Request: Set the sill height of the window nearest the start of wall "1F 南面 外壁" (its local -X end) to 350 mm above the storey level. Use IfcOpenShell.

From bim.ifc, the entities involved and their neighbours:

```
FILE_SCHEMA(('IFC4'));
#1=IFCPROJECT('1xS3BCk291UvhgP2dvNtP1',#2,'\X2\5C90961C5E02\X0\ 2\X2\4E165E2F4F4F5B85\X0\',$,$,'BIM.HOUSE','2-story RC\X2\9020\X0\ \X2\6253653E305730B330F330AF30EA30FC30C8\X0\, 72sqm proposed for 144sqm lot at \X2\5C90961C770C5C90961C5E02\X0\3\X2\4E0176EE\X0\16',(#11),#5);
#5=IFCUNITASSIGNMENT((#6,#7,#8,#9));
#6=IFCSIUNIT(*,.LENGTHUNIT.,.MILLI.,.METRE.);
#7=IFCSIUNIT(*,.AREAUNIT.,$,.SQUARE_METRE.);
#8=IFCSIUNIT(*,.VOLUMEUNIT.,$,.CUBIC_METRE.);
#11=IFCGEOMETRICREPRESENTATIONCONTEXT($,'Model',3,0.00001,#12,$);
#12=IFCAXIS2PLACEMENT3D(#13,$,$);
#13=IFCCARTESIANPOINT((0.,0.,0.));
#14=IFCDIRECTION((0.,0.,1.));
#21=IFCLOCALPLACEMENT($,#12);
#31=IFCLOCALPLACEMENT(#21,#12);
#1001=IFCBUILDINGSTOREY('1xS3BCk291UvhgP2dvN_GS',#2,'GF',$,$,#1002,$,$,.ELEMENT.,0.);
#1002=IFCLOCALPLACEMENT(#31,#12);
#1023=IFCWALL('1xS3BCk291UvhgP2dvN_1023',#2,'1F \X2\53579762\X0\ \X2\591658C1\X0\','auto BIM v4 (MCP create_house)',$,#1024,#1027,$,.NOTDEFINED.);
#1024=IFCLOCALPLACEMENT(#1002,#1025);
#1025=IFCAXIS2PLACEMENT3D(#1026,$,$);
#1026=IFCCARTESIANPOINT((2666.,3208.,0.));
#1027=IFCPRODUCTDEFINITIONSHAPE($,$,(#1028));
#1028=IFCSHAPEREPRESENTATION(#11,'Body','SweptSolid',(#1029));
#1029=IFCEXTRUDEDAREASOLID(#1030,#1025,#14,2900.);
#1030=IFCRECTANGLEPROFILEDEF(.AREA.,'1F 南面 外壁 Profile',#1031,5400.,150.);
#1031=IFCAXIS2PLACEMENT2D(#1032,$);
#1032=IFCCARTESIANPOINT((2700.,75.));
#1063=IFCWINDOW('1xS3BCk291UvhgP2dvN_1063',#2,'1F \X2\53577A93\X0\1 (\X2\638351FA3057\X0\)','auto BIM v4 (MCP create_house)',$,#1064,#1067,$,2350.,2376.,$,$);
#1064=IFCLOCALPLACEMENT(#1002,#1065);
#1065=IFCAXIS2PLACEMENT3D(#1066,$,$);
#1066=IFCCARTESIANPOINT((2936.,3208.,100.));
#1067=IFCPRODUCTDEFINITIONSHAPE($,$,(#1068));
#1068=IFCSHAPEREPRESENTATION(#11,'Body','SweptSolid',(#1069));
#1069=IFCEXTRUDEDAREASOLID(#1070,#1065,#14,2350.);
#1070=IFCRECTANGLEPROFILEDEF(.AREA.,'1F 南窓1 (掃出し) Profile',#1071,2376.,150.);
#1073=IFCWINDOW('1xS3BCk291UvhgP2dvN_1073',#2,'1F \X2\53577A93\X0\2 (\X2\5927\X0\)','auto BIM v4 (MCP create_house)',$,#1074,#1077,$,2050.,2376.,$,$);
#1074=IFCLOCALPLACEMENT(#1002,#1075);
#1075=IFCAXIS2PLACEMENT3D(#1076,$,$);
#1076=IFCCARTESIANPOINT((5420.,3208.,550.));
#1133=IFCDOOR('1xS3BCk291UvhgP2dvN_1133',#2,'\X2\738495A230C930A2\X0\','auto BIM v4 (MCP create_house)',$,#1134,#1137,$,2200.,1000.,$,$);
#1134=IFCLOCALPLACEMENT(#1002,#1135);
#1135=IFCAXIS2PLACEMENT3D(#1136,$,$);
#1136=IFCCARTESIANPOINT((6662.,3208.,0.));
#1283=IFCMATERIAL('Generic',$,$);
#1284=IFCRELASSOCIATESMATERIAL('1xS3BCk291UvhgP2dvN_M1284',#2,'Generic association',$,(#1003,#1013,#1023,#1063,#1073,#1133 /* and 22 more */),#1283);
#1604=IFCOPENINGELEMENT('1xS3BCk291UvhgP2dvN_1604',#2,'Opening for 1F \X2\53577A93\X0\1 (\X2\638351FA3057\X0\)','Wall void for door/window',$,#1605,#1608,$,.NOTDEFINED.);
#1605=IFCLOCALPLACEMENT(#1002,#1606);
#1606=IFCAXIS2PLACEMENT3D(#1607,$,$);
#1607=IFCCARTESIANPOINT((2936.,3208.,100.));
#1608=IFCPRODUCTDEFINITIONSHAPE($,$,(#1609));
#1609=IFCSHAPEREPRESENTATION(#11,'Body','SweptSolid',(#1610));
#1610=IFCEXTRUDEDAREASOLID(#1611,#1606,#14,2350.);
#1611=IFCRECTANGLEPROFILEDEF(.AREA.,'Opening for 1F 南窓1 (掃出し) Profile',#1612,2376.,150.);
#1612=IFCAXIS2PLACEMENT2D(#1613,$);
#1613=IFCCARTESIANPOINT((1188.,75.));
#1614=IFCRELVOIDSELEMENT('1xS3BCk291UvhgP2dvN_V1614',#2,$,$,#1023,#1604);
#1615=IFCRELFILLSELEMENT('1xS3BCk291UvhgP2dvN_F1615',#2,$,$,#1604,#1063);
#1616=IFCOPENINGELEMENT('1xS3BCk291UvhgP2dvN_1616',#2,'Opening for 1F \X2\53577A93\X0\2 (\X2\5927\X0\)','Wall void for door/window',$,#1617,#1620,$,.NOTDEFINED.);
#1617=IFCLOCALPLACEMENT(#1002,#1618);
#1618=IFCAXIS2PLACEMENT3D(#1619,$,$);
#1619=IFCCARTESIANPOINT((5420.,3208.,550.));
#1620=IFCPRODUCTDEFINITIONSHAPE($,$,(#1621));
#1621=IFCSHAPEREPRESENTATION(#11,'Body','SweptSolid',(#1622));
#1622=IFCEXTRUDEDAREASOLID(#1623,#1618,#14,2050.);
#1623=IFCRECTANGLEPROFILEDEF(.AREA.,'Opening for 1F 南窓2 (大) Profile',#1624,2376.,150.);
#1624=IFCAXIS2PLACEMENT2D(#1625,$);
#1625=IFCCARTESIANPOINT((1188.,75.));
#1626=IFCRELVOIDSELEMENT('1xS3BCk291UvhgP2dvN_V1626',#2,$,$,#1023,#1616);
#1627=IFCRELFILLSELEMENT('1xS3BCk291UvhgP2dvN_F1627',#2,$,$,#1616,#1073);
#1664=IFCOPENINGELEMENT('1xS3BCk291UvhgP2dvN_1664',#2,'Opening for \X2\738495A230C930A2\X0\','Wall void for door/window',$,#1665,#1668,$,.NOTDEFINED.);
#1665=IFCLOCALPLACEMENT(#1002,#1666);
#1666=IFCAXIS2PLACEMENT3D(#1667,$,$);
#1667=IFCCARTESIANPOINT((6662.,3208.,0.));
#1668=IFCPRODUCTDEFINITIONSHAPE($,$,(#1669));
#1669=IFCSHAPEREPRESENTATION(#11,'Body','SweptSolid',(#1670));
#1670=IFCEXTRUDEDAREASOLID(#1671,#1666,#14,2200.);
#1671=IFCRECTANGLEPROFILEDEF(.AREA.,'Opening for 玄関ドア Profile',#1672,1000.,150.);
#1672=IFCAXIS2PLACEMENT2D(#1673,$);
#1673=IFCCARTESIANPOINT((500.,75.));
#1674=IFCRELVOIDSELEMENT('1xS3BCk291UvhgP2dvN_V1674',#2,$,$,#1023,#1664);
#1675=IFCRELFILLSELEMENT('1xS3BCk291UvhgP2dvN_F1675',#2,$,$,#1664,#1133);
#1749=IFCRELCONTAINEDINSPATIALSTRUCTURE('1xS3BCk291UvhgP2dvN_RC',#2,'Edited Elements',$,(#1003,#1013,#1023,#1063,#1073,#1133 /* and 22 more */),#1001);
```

```python
import numpy as np
import ifcopenshell
import ifcopenshell.api.geometry
import ifcopenshell.geom
import ifcopenshell.util.element
import ifcopenshell.util.placement
import ifcopenshell.util.shape
import ifcopenshell.util.unit

model = ifcopenshell.open("bim.ifc")
unit_scale = ifcopenshell.util.unit.calculate_unit_scale(model)

window = model.by_guid("1xS3BCk291UvhgP2dvN_1063")
opening = window.FillsVoids[0].RelatingOpeningElement
storey = ifcopenshell.util.element.get_container(window, ifc_class="IfcBuildingStorey")
level = ifcopenshell.util.placement.get_local_placement(storey.ObjectPlacement)[2, 3]

# The opening's origin need not be at the sill, so measure its lowest point.
shape = ifcopenshell.geom.create_shape(ifcopenshell.geom.settings(), opening)
bottom = ifcopenshell.util.shape.get_shape_bottom_elevation(shape, shape.geometry) / unit_scale
dz = level + 350.0 - bottom

shift = np.array([0.0, 0.0, dz])
# The window is not placed relative to its opening, so move both.
for product in (opening, window):
    matrix = ifcopenshell.util.placement.get_local_placement(product.ObjectPlacement)
    matrix[:3, 3] += shift
    ifcopenshell.api.geometry.edit_object_placement(model, product=product, matrix=matrix, is_si=False)

print(f"moved by {dz * unit_scale:+.3f} m")

model.write("bim_edited.ifc")
```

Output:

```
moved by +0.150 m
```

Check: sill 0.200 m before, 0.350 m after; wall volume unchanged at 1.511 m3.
